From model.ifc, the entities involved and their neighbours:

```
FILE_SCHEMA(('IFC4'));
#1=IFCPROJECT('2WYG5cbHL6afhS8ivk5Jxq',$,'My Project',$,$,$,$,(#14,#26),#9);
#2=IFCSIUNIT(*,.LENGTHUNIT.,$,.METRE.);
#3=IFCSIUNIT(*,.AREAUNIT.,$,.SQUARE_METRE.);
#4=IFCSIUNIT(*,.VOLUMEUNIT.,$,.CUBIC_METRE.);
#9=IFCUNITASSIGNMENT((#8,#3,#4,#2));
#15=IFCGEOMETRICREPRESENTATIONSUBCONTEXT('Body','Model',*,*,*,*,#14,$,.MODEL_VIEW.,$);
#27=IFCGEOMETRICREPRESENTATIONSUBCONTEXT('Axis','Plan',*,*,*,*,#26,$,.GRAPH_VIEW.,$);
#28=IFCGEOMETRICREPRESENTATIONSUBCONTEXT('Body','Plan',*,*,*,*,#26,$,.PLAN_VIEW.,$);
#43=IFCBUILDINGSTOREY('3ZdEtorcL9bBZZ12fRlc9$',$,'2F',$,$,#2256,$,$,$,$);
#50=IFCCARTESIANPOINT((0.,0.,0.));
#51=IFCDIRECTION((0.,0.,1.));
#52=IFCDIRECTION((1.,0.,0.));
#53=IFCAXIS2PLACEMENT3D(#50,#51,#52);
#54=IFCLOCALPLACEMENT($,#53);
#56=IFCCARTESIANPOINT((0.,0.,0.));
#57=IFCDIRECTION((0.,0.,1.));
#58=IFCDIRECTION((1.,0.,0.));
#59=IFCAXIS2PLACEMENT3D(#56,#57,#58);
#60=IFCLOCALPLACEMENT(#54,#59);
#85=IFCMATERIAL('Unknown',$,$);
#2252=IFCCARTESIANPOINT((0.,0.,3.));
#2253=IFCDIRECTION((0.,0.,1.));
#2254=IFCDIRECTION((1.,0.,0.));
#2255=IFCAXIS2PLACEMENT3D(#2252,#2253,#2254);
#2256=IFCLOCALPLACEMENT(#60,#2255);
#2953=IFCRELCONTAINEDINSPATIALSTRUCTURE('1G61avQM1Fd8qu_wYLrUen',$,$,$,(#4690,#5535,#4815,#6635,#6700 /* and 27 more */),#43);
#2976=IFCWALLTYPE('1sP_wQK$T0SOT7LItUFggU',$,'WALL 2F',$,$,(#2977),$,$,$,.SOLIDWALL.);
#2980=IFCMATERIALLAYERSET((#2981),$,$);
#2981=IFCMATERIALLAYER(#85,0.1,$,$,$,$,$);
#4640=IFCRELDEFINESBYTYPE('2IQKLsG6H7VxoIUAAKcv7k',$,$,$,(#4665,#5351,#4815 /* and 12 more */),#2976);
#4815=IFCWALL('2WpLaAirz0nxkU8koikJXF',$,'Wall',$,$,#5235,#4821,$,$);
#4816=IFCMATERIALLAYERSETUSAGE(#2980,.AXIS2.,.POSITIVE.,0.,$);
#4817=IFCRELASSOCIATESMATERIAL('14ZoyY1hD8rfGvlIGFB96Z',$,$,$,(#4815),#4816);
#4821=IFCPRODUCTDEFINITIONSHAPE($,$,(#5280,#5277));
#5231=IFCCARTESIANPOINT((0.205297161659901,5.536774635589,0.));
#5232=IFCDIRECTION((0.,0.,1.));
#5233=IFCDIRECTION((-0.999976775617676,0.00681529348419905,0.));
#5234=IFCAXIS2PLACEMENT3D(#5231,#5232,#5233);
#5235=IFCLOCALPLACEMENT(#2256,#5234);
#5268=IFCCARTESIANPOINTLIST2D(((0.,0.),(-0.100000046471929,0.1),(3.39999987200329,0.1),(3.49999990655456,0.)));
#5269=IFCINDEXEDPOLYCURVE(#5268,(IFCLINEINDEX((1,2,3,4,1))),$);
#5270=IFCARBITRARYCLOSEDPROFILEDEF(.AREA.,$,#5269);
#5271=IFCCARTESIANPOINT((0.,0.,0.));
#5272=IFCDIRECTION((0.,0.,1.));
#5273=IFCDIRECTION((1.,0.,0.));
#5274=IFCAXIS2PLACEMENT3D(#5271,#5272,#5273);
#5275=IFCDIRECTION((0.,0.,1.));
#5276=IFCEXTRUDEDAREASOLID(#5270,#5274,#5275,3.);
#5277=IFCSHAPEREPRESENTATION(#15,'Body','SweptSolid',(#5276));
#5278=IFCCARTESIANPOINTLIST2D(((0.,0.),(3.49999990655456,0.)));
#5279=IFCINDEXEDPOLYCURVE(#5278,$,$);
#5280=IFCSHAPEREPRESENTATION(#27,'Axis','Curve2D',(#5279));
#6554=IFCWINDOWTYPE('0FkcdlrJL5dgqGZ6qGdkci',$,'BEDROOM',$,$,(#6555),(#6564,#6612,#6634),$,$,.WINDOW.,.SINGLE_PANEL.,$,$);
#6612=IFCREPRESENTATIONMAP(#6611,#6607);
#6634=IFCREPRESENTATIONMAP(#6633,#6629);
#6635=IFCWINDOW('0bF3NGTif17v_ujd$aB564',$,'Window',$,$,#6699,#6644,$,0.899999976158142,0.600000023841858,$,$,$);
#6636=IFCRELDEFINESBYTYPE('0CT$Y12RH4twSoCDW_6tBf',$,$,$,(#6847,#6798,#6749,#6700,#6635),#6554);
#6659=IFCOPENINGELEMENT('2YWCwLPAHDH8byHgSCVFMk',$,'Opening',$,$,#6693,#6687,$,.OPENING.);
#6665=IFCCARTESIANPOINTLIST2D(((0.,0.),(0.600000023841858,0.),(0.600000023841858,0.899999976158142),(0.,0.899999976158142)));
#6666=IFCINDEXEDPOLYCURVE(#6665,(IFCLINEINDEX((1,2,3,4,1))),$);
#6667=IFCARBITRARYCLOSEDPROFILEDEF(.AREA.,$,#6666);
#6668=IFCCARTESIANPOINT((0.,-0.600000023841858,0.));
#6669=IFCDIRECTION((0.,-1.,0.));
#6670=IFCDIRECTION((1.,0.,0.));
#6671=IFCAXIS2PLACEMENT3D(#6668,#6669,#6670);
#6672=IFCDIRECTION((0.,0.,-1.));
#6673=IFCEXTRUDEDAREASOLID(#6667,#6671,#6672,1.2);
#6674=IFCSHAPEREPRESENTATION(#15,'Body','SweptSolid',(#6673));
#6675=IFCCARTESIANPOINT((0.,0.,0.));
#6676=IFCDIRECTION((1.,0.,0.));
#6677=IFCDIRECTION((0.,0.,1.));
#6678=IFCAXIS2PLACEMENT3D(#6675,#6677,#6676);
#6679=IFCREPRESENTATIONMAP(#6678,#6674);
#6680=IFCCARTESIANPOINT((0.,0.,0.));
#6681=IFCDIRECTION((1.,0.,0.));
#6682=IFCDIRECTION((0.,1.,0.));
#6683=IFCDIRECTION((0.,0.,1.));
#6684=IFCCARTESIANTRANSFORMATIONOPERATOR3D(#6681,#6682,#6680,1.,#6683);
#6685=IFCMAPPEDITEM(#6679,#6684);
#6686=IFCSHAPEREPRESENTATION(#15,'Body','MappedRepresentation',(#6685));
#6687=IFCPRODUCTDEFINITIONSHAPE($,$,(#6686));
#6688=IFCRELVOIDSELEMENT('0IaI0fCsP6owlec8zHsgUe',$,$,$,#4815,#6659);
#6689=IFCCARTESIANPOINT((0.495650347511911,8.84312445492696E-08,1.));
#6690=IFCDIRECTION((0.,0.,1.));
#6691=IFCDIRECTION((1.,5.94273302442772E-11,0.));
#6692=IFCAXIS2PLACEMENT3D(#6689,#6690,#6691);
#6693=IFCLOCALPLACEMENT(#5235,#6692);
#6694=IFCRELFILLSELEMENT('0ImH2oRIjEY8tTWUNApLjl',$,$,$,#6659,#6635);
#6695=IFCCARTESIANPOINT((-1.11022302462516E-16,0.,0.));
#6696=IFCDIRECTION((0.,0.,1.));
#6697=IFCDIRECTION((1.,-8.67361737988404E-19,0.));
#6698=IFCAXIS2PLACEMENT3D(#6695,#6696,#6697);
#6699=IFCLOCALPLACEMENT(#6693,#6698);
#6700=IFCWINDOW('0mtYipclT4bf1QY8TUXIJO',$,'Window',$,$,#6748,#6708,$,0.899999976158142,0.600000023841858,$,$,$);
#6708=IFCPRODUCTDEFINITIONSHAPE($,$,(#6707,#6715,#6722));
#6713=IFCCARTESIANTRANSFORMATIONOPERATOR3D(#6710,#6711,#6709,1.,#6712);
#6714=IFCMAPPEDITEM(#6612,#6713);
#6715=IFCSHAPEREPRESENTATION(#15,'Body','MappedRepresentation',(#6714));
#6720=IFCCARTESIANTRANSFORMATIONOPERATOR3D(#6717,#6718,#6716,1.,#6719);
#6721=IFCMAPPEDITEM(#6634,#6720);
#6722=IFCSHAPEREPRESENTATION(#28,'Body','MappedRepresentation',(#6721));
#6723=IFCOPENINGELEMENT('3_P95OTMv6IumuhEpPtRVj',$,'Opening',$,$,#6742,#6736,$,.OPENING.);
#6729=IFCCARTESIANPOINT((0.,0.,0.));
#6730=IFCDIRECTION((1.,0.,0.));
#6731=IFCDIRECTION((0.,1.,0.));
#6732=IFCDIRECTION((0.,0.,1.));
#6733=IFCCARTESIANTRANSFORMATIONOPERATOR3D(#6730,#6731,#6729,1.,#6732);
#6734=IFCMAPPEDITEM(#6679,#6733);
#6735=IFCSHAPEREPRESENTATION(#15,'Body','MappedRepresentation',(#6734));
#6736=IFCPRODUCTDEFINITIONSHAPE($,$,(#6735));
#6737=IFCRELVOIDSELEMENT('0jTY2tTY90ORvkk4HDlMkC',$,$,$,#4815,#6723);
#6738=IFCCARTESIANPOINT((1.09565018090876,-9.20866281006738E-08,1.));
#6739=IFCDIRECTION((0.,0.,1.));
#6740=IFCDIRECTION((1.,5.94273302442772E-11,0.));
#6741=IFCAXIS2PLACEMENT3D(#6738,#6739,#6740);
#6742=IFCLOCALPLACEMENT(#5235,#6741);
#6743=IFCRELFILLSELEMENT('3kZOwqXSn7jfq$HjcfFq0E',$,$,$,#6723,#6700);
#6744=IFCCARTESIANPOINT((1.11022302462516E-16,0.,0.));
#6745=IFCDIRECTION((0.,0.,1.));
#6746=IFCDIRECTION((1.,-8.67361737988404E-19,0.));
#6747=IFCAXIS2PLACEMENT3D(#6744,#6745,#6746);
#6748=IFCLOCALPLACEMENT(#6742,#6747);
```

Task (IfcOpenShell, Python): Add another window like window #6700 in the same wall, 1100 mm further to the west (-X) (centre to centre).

```python
import ifcopenshell
import ifcopenshell.api.feature
import ifcopenshell.api.geometry
import ifcopenshell.api.root
import ifcopenshell.geom
import ifcopenshell.util.element
import ifcopenshell.util.placement
import ifcopenshell.util.shape
import ifcopenshell.util.unit

model = ifcopenshell.open("model.ifc")
unit_scale = ifcopenshell.util.unit.calculate_unit_scale(model)
settings = ifcopenshell.geom.settings()


def volume(element):
    """Net volume in cubic metres, openings subtracted."""
    shape = ifcopenshell.geom.create_shape(settings, element)
    return ifcopenshell.util.shape.get_volume(shape.geometry)


window = model.by_guid("0mtYipclT4bf1QY8TUXIJO")
opening = window.FillsVoids[0].RelatingOpeningElement
wall = opening.VoidsElements[0].RelatingBuildingElement
before = volume(wall)
shift = ifcopenshell.util.placement.get_local_placement(wall.ObjectPlacement)[:3, 0] * 1.1 / unit_scale

# copy_class copies the void relationship, type, container and properties, but no geometry.
new_opening = ifcopenshell.api.root.copy_class(model, product=opening)
new_opening.Representation = ifcopenshell.util.element.copy_deep(
    model, opening.Representation, exclude=["IfcGeometricRepresentationContext", "IfcRepresentationMap"]
)
new_window = ifcopenshell.api.root.copy_class(model, product=window)
new_window.Representation = ifcopenshell.util.element.copy_deep(
    model, window.Representation, exclude=["IfcGeometricRepresentationContext", "IfcRepresentationMap"]
)
ifcopenshell.api.feature.add_filling(model, opening=new_opening, element=new_window)

for old, new in ((opening, new_opening), (window, new_window)):
    matrix = ifcopenshell.util.placement.get_local_placement(old.ObjectPlacement)
    matrix[:3, 3] += shift
    ifcopenshell.api.geometry.edit_object_placement(model, product=new, matrix=matrix, is_si=False)

after = volume(wall)

print(f"wall volume {before:.3f} -> {after:.3f} m3")

model.write("model_rev.ifc")
```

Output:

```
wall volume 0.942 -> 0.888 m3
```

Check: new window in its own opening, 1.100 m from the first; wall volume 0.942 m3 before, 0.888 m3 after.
